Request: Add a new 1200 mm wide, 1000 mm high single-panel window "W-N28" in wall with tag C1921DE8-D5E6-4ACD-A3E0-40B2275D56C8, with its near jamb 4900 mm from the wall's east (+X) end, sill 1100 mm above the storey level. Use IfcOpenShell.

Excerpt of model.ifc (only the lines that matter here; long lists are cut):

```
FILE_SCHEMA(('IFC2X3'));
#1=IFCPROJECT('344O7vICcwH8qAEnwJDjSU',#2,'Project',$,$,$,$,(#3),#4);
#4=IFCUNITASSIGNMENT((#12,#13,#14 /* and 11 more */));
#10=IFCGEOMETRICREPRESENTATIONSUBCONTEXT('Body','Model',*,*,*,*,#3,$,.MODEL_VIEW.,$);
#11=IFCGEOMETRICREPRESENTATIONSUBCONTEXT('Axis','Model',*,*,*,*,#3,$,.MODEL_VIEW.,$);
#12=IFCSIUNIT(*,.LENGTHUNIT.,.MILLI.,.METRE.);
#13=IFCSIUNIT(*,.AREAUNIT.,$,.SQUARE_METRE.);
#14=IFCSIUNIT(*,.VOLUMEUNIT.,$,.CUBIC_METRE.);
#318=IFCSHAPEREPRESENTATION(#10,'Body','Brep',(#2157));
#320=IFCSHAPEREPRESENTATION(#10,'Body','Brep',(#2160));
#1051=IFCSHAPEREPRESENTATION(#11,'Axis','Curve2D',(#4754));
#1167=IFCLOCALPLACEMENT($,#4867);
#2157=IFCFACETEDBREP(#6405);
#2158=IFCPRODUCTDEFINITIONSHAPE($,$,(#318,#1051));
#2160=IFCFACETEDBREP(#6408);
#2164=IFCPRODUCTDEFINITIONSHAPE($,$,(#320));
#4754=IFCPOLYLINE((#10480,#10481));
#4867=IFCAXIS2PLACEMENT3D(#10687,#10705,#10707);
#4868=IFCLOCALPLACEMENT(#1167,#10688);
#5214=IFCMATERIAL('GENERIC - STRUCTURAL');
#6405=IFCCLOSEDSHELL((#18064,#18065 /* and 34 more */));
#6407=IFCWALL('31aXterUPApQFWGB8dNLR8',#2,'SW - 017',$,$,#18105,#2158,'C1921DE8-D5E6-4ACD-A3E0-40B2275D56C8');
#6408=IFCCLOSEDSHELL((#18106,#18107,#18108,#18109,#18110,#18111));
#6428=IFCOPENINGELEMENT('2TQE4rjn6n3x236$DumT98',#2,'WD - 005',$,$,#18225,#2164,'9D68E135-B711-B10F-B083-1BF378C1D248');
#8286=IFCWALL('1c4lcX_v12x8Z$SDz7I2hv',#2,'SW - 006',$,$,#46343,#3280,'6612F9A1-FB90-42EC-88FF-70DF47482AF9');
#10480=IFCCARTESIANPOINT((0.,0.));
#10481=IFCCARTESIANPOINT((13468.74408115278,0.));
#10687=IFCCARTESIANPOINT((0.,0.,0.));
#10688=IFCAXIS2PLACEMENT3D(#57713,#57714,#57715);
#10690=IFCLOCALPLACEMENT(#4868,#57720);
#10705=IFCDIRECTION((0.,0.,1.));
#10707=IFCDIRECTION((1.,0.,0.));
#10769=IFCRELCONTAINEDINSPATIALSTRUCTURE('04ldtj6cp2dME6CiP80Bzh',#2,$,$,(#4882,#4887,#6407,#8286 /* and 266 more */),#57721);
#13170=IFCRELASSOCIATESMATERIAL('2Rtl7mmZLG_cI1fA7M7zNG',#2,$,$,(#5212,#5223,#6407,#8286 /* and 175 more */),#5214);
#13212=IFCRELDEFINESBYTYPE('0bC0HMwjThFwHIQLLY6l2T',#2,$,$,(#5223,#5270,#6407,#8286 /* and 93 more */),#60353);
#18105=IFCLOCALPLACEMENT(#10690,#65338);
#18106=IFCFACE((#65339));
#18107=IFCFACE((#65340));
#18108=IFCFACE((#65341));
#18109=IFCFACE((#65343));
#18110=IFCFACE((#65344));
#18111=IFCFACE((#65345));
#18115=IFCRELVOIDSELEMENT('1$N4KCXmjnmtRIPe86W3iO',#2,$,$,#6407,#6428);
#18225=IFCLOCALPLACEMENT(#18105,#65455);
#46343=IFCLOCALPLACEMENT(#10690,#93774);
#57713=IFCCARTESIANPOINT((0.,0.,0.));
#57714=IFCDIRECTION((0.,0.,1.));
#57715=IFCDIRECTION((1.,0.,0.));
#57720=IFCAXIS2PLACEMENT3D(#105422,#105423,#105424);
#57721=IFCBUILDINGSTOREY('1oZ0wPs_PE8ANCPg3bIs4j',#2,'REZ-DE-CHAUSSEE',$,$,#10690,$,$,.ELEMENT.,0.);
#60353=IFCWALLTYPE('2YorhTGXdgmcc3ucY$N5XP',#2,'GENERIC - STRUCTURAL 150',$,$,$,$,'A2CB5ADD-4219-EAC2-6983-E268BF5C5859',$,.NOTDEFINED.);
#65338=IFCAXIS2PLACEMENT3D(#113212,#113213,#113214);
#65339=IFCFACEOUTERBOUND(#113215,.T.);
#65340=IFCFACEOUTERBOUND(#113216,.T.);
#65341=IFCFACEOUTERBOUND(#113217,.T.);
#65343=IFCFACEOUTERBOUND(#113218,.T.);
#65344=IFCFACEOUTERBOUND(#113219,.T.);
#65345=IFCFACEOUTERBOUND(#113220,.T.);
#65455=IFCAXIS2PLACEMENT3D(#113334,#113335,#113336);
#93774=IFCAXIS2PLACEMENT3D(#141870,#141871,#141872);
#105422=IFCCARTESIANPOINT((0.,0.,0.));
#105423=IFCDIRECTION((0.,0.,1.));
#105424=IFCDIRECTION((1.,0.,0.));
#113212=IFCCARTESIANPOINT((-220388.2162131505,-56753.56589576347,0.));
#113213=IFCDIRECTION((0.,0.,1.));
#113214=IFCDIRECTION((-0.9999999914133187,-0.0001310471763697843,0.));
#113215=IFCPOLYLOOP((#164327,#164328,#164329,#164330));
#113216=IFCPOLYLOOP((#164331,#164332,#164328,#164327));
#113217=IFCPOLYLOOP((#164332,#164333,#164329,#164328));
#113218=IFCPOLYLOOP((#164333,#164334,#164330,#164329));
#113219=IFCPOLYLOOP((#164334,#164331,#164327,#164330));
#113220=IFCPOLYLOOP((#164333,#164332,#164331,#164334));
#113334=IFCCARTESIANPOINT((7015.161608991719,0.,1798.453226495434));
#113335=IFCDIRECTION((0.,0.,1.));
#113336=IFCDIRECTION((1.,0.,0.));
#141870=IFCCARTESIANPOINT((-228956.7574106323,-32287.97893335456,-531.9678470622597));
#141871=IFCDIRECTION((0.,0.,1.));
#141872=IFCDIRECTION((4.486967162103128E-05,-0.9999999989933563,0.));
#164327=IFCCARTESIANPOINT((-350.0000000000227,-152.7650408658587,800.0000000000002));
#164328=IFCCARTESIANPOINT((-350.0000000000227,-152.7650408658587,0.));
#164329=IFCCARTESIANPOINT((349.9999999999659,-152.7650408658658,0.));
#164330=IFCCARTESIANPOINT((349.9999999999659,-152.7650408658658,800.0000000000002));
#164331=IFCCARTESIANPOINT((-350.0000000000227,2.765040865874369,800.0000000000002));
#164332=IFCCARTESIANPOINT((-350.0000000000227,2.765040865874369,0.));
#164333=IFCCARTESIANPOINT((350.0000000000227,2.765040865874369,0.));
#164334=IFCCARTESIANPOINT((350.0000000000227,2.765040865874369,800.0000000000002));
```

```python
import numpy as np
import ifcopenshell
import ifcopenshell.api.feature
import ifcopenshell.api.geometry
import ifcopenshell.api.root
import ifcopenshell.api.spatial
import ifcopenshell.api.type
import ifcopenshell.geom
import ifcopenshell.util.element
import ifcopenshell.util.placement
import ifcopenshell.util.representation
import ifcopenshell.util.shape
import ifcopenshell.util.unit

model = ifcopenshell.open("model.ifc")
unit_scale = ifcopenshell.util.unit.calculate_unit_scale(model)
settings = ifcopenshell.geom.settings()


def volume(element):
    """Net volume in cubic metres, openings subtracted."""
    shape = ifcopenshell.geom.create_shape(settings, element)
    return ifcopenshell.util.shape.get_volume(shape.geometry)


wall = model.by_guid("31aXterUPApQFWGB8dNLR8")
storey = ifcopenshell.util.element.get_container(wall, ifc_class="IfcBuildingStorey")
context = ifcopenshell.util.representation.get_context(model, "Model", "Body", "MODEL_VIEW")
before = volume(wall)

width, height, from_end, sill = 1.2, 1, 4.9, 1.1  # metres

# The wall runs along its own X axis, and the end named is its -X end.
wall_shape = ifcopenshell.geom.create_shape(settings, wall)
x, y, z = ifcopenshell.util.shape.get_vertices(wall_shape.geometry).T
start = x.min() + from_end
face, thickness = float(y.min()), float(y.max() - y.min())
wall_matrix = ifcopenshell.util.placement.get_local_placement(wall.ObjectPlacement)
level = ifcopenshell.util.placement.get_local_placement(storey.ObjectPlacement)[2, 3]


def in_wall(x, y):
    """Placement at x, y metres in the wall's axes, at sill height."""
    matrix = wall_matrix.copy()
    matrix[:, 3] = wall_matrix @ np.array([x / unit_scale, y / unit_scale, 0.0, 1.0])
    matrix[2, 3] = level + sill / unit_scale
    return matrix


# Opening: a box that overshoots both wall faces by 50 mm.
opening = ifcopenshell.api.root.create_entity(model, ifc_class="IfcOpeningElement")
box = ifcopenshell.api.geometry.add_wall_representation(
    model, context=context, length=width, height=height, thickness=thickness + 0.1
)
ifcopenshell.api.geometry.assign_representation(model, product=opening, representation=box)
ifcopenshell.api.geometry.edit_object_placement(model, product=opening, matrix=in_wall(start, face - 0.05), is_si=False)
ifcopenshell.api.feature.add_feature(model, feature=opening, element=wall)

window = ifcopenshell.api.root.create_entity(model, ifc_class="IfcWindow", name="W-N28")
window.OverallWidth, window.OverallHeight = width / unit_scale, height / unit_scale
body = ifcopenshell.api.geometry.add_window_representation(
    model,
    context=context,
    overall_width=window.OverallWidth,
    overall_height=window.OverallHeight,
    partition_type="SINGLE_PANEL",
)
ifcopenshell.api.geometry.assign_representation(model, product=window, representation=body)
ifcopenshell.api.spatial.assign_container(model, products=[window], relating_structure=storey)
fills = ifcopenshell.api.feature.add_filling(model, opening=opening, element=window)
fills.OwnerHistory = window.OwnerHistory  # required in IFC2X3

# IFC2X3 keeps the operation on the window style.
style = ifcopenshell.api.root.create_entity(model, ifc_class="IfcWindowStyle", name="W-N28")
style.OperationType, style.ConstructionType = "SINGLE_PANEL", "NOTDEFINED"
style.ParameterTakesPrecedence = style.Sizeable = False
ifcopenshell.api.type.assign_type(model, related_objects=[window], relating_type=style)

# Centre the window in the wall's thickness.
ifcopenshell.api.geometry.edit_object_placement(model, product=window, matrix=in_wall(start, face), is_si=False)
window_shape = ifcopenshell.geom.create_shape(settings, window)
depth = ifcopenshell.util.shape.get_vertices(window_shape.geometry)[:, 1]
offset = face + thickness / 2 - (depth.min() + depth.max()) / 2
ifcopenshell.api.geometry.edit_object_placement(model, product=window, matrix=in_wall(start, offset), is_si=False)

after = volume(wall)

print(f"wall volume {before:.3f} -> {after:.3f} m3")

model.write("model-out.ifc")
```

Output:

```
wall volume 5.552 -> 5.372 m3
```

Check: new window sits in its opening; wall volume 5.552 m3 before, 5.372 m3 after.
